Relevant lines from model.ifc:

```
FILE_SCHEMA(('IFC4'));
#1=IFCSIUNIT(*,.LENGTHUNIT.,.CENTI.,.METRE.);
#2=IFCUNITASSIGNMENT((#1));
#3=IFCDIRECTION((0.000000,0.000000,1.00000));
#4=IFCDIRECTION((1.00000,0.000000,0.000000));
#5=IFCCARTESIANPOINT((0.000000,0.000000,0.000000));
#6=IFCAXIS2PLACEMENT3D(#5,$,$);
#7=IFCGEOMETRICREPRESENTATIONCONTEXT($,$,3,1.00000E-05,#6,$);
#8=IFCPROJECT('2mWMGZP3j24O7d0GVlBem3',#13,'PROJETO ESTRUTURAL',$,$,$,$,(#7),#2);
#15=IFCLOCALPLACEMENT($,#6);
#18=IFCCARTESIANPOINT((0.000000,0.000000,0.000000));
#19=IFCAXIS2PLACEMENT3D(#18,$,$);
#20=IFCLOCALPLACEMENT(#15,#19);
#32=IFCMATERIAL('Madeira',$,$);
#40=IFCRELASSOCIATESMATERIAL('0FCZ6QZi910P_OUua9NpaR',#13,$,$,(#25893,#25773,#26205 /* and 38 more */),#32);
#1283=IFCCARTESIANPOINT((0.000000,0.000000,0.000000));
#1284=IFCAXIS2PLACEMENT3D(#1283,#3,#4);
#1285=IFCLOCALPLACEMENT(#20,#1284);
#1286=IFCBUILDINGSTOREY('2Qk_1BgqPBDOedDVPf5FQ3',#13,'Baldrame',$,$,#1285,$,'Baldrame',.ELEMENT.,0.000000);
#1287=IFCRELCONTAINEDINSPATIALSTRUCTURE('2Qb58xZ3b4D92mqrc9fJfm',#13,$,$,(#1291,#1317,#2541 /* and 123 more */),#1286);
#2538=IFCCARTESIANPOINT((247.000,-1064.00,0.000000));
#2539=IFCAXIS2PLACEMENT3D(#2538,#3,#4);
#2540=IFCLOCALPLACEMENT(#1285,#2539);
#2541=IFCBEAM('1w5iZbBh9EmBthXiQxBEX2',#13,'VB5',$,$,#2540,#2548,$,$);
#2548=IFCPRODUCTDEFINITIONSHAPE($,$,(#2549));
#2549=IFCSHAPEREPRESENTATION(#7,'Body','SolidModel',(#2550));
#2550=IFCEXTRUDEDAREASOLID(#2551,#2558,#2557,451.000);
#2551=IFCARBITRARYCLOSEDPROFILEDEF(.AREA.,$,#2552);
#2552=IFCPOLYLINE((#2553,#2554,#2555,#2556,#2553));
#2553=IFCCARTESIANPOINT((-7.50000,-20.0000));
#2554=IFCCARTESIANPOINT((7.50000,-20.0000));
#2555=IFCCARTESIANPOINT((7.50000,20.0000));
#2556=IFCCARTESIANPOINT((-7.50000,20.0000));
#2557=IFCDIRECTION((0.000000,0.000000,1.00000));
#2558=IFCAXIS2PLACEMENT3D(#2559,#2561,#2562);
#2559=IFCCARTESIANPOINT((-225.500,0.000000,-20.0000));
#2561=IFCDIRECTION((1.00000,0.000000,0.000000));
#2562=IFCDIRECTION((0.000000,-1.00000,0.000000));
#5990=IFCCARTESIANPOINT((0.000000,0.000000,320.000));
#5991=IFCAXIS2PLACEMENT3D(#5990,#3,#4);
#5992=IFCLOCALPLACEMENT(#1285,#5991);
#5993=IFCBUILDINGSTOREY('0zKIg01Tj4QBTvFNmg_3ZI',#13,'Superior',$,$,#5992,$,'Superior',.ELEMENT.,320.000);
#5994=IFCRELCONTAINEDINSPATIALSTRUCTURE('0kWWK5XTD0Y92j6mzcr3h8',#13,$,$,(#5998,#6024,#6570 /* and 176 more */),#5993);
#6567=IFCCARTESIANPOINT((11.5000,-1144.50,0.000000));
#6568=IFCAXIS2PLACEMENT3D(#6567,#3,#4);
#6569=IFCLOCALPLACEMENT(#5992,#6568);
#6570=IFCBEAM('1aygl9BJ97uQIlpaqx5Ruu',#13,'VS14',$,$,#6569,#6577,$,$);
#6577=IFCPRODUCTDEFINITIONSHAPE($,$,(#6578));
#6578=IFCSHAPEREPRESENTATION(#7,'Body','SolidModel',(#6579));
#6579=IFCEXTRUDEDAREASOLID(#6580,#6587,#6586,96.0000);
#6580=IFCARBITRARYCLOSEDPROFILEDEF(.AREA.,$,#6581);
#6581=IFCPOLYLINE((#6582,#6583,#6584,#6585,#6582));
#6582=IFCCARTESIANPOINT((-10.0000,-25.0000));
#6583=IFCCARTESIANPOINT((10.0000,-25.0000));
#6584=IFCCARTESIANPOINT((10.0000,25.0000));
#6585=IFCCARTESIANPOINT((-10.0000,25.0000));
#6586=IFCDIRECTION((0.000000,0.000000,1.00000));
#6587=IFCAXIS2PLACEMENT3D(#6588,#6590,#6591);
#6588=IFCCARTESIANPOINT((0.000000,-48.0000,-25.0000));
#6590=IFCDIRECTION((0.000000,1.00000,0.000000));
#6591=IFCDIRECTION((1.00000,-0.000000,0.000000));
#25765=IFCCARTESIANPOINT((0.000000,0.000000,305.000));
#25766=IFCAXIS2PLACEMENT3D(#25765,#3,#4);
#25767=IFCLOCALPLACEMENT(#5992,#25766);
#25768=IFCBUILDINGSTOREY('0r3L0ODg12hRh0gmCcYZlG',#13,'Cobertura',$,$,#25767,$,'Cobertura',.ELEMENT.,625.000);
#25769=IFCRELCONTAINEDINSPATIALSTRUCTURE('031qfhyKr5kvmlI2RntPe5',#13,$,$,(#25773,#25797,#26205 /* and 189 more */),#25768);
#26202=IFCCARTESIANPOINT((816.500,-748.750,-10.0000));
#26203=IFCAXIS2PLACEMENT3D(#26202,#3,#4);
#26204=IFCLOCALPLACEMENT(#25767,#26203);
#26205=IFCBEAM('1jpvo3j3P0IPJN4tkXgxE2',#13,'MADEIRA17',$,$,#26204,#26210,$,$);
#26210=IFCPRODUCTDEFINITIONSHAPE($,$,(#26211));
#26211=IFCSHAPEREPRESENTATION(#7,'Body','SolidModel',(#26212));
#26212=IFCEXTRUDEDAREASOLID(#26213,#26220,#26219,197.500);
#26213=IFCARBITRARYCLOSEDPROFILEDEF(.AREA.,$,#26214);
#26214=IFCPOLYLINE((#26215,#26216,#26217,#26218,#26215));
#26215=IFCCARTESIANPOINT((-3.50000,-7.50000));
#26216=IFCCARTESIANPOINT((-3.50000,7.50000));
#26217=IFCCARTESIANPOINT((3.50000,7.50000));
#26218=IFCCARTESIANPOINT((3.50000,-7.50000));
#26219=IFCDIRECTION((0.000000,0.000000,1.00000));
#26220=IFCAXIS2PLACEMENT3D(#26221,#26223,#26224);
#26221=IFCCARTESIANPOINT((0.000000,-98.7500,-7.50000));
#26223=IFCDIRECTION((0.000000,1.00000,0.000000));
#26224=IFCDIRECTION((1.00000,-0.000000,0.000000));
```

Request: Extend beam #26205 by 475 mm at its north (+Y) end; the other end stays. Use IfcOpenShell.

```python
import ifcopenshell
import ifcopenshell.util.unit

model = ifcopenshell.open("model.ifc")
unit_scale = ifcopenshell.util.unit.calculate_unit_scale(model)

member = model.by_guid("1jpvo3j3P0IPJN4tkXgxE2")
change = 0.475 / unit_scale

# The extrusion runs towards the end named, so only its depth changes.
body = next(r for r in member.Representation.Representations if r.RepresentationIdentifier == "Body")
solid = body.Items[0]
old_length = solid.Depth
solid.Depth += change

print(f"length {old_length:g} -> {solid.Depth:g}")

model.write("model_updated.ifc")
```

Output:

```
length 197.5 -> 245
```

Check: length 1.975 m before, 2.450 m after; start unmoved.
